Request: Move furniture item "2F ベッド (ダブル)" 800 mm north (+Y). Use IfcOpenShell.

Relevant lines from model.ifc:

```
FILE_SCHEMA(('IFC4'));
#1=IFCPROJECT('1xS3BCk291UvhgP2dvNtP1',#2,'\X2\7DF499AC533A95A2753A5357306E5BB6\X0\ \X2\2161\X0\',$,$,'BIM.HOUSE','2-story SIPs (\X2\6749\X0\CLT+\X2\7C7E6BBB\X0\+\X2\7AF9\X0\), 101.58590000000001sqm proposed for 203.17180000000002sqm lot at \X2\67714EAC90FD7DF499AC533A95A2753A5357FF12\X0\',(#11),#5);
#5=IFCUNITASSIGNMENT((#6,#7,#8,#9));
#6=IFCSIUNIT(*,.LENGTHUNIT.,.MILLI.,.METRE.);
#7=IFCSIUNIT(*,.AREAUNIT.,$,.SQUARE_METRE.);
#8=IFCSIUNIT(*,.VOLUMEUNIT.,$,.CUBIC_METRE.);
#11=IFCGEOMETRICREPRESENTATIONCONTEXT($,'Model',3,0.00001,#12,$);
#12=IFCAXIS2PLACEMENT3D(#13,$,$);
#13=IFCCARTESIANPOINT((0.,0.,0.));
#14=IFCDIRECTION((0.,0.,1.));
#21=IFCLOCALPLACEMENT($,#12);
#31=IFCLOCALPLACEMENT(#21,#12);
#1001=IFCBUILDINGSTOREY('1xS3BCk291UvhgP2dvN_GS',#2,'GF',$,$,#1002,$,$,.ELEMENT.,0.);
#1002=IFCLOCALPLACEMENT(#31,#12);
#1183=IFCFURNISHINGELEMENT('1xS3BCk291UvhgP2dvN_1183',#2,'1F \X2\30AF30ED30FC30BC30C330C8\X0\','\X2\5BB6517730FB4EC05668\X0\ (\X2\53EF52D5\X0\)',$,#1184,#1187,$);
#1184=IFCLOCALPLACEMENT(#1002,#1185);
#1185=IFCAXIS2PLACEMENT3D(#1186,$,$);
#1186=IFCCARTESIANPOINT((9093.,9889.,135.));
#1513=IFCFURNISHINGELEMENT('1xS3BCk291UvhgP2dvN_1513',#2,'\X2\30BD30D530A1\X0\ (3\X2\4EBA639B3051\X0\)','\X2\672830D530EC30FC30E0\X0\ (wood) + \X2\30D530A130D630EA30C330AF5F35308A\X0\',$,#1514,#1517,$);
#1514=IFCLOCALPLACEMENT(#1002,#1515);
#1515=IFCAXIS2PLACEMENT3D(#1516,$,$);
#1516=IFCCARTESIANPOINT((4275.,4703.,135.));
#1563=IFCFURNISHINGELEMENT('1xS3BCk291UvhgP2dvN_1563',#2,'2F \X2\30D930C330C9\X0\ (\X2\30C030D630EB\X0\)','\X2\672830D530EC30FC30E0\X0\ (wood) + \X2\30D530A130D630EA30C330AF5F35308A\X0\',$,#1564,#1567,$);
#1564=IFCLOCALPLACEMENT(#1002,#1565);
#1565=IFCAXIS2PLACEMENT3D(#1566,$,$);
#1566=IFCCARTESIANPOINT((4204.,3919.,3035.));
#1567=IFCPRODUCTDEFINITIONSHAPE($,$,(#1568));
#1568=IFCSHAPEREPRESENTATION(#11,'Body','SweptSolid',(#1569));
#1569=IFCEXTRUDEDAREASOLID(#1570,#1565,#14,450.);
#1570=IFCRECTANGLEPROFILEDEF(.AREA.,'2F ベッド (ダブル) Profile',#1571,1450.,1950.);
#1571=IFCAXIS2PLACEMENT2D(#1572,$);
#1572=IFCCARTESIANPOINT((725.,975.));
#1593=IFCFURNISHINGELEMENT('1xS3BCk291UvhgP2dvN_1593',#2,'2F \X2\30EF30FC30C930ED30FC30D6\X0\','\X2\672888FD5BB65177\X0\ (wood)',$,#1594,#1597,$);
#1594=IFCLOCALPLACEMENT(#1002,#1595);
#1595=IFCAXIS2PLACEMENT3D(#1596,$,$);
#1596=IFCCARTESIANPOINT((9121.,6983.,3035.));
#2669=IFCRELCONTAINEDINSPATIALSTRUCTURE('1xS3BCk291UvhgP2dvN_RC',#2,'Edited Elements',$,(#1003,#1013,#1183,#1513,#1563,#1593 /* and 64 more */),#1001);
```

```python
import ifcopenshell
import ifcopenshell.api.geometry
import ifcopenshell.util.placement

model = ifcopenshell.open("model.ifc")

item = model.by_id(1563)
matrix = ifcopenshell.util.placement.get_local_placement(item.ObjectPlacement)
matrix[1, 3] += 800.0
ifcopenshell.api.geometry.edit_object_placement(model, product=item, matrix=matrix, is_si=False)

print(ifcopenshell.util.placement.get_local_placement(item.ObjectPlacement).round(3) + 0.0)

model.write("model_rev.ifc")
```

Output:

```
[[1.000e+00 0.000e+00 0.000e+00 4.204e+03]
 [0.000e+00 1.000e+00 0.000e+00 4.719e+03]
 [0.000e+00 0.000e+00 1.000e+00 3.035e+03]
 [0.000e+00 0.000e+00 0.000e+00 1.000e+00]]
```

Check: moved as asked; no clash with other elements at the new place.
